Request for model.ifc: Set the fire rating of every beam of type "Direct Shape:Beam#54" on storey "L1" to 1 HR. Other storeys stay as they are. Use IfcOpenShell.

First a look at what the model holds.

```python
import ifcopenshell
import ifcopenshell.util.element

model = ifcopenshell.open("model.ifc")
print(model.schema)
storey = next(s for s in model.by_type("IfcBuildingStorey") if s.Name == "L1")
beams = [e for e in ifcopenshell.util.element.get_decomposition(storey) if e.is_a("IfcBeam")]
seen = {}
for e in beams:
    element_type = ifcopenshell.util.element.get_type(e)
    key = (element_type.Name if element_type != e and element_type else None, ifcopenshell.util.element.get_pset(e, "Pset_BeamCommon", "FireRating"))
    seen[key] = seen.get(key, 0) + 1
for (name, value), count in sorted(seen.items(), key=str):
    print(count, "x", name, "|", value)
```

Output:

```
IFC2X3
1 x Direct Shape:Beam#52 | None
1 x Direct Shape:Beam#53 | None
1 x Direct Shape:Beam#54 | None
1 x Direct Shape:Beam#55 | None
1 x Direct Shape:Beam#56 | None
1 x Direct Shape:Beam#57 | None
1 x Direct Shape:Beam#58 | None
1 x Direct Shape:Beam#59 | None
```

```python
import ifcopenshell
import ifcopenshell.api.pset
import ifcopenshell.util.element

model = ifcopenshell.open("model.ifc")

storey = next(s for s in model.by_type("IfcBuildingStorey") if s.Name == "L1")
beams = [e for e in ifcopenshell.util.element.get_decomposition(storey) if e.is_a("IfcBeam")]

count = 0
for e in beams:
    element_type = ifcopenshell.util.element.get_type(e)
    if element_type in (None, e) or element_type.Name != "Direct Shape:Beam#54":
        continue
    # add_pset returns the element's existing set when there is one.
    pset = ifcopenshell.api.pset.add_pset(model, product=e, name="Pset_BeamCommon")
    ifcopenshell.api.pset.edit_pset(model, pset=pset, properties={"FireRating": "1 HR"})
    count += 1

print(count, "beams updated")

model.write("model_edited.ifc")
```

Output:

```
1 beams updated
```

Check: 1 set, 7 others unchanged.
